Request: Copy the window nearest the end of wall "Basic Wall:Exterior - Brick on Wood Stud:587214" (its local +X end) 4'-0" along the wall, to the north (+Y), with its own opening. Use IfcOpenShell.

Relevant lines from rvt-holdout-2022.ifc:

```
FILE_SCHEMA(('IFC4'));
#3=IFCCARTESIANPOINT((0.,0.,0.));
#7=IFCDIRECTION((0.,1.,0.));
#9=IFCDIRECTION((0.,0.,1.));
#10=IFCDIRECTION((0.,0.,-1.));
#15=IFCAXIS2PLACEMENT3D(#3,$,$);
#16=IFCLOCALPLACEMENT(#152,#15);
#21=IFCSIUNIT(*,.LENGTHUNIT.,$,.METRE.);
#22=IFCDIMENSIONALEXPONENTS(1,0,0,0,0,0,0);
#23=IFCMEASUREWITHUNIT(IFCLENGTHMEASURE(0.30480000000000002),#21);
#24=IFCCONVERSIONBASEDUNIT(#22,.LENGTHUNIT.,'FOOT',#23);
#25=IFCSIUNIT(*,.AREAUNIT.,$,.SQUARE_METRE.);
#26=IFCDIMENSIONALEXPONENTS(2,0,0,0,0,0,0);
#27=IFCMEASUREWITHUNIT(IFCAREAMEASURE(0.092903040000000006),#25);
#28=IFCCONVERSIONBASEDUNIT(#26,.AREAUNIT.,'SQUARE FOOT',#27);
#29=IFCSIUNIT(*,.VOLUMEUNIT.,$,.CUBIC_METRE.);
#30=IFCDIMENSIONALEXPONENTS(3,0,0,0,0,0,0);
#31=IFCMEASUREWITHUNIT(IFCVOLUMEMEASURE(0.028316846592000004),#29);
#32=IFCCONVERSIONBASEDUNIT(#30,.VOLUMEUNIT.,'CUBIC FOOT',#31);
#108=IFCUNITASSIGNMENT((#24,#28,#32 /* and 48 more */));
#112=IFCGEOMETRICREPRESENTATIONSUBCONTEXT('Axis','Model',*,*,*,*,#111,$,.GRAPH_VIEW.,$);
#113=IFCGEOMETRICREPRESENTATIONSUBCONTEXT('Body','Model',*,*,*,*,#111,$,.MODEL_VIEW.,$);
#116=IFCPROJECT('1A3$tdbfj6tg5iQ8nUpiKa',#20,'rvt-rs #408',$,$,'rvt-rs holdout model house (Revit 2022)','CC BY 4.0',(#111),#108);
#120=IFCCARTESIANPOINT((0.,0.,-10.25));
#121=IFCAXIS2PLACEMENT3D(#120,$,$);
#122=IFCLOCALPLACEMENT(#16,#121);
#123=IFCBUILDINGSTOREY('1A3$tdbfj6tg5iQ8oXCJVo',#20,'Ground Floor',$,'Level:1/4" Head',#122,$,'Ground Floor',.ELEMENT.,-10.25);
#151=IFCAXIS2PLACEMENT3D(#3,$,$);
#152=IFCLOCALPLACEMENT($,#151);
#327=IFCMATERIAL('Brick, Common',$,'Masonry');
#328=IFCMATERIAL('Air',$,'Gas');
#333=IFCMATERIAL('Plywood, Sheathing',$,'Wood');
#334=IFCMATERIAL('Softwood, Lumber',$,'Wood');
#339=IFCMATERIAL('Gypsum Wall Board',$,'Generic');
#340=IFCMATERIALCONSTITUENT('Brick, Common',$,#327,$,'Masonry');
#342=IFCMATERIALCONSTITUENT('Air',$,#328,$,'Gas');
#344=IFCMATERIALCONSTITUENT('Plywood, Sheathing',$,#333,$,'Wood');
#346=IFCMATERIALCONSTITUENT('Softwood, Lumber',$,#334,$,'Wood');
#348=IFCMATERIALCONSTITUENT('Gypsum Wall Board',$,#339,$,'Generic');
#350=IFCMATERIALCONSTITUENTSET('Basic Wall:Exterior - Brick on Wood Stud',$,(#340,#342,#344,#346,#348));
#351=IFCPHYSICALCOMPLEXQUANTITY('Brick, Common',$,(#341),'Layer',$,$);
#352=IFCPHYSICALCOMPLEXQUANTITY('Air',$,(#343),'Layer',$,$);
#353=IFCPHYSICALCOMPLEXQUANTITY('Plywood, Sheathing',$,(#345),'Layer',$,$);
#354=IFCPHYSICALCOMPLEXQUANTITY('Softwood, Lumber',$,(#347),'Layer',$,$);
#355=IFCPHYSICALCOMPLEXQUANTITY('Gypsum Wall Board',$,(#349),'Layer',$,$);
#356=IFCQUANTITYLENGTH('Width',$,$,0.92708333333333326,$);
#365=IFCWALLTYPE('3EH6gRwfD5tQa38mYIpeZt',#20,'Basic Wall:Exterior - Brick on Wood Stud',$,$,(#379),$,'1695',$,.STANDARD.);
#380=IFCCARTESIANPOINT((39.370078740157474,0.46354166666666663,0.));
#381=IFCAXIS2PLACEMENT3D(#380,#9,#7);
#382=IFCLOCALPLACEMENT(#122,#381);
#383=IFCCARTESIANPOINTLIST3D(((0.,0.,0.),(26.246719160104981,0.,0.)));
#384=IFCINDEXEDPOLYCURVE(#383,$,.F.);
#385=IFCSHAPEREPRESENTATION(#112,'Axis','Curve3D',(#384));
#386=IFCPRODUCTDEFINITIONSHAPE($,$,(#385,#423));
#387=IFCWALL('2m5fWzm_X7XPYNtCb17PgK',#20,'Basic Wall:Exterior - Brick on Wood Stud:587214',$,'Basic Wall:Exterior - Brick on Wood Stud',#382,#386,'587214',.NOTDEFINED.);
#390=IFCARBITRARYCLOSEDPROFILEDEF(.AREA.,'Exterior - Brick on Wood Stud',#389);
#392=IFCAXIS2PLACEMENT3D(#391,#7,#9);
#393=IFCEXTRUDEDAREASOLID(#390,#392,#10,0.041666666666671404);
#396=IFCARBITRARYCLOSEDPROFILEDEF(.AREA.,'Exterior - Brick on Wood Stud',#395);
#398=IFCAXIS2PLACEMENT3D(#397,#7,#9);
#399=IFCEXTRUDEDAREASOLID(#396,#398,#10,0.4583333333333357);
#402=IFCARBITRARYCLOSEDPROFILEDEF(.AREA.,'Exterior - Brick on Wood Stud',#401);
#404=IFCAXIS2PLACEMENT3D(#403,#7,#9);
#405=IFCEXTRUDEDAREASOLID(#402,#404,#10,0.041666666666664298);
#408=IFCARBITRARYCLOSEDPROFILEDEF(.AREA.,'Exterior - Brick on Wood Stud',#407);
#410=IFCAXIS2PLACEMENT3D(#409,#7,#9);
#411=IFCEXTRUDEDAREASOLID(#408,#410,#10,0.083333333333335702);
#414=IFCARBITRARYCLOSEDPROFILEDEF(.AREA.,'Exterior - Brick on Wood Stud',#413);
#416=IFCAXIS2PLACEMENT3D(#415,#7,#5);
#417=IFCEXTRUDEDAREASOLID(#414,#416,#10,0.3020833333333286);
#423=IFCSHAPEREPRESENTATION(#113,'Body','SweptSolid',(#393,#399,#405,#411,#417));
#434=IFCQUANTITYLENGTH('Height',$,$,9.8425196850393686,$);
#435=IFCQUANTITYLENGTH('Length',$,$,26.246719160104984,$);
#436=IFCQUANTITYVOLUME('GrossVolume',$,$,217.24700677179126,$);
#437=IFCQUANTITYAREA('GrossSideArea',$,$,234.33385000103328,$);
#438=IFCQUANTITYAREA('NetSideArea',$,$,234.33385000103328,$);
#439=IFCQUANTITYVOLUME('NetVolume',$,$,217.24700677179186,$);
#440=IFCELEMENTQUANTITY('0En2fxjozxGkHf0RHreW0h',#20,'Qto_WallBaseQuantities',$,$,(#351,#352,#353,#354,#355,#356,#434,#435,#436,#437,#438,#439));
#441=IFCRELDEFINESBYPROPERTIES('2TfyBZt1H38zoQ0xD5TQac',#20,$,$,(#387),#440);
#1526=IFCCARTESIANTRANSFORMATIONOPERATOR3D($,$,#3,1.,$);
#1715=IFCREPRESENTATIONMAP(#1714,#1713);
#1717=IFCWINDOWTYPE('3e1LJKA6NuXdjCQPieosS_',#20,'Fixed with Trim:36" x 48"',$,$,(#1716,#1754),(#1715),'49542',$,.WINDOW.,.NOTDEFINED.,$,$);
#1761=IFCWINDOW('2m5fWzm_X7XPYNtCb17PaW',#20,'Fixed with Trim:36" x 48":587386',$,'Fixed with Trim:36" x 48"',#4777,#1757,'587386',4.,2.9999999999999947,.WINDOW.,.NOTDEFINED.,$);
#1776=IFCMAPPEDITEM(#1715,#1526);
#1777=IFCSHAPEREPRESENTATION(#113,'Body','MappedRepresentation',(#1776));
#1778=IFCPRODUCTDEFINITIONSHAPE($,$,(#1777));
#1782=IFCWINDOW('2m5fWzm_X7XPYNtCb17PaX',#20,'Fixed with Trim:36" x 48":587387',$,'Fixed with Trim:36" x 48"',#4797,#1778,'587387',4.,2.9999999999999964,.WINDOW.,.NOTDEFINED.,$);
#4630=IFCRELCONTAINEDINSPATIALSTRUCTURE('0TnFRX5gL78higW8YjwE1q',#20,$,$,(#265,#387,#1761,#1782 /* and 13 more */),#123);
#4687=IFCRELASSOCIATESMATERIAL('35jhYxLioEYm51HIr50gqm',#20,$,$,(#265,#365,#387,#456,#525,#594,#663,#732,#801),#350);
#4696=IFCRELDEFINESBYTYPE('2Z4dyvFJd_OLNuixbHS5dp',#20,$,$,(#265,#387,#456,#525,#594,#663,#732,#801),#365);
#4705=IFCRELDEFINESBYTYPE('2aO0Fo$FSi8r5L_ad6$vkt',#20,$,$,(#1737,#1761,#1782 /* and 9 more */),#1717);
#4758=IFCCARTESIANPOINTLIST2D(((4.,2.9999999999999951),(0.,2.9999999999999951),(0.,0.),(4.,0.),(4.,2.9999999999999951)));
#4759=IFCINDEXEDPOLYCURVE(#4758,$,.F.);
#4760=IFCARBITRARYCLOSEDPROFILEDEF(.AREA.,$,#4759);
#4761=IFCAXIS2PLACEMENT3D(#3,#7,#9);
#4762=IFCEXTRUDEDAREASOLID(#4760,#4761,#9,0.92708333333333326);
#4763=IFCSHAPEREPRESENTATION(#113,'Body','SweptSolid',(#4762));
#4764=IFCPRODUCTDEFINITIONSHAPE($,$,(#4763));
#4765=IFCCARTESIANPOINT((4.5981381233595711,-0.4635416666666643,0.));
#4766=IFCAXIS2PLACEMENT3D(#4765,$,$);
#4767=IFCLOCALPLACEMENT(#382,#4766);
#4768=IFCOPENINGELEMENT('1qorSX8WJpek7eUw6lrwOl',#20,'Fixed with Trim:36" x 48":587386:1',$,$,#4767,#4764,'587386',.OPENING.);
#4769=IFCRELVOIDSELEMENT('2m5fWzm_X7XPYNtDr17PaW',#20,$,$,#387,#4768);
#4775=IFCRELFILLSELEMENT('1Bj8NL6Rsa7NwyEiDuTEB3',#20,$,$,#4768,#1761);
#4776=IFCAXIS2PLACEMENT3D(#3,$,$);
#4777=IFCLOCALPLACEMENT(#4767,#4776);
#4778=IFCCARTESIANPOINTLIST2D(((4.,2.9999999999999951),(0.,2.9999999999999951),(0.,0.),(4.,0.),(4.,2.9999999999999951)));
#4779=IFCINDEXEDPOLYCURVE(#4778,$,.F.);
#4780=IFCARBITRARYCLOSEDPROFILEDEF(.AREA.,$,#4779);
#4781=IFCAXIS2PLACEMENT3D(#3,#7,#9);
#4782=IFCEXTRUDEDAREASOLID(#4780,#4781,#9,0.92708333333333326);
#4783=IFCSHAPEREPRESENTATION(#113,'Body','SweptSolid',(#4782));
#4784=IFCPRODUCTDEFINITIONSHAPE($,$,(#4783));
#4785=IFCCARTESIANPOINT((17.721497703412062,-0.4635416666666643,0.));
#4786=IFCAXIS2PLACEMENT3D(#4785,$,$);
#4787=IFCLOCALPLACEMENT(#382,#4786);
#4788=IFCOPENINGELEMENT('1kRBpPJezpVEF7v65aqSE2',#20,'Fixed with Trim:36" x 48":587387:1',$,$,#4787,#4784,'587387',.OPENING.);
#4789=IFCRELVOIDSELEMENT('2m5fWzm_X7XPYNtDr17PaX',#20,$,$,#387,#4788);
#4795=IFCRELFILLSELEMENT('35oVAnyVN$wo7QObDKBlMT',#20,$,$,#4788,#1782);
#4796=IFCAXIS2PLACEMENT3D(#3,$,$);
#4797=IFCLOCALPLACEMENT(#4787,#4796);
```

```python
import ifcopenshell
import ifcopenshell.api.feature
import ifcopenshell.api.geometry
import ifcopenshell.api.pset
import ifcopenshell.api.root
import ifcopenshell.geom
import ifcopenshell.util.element
import ifcopenshell.util.placement
import ifcopenshell.util.shape
import ifcopenshell.util.unit

model = ifcopenshell.open("rvt-holdout-2022.ifc")
unit_scale = ifcopenshell.util.unit.calculate_unit_scale(model)
area_scale = ifcopenshell.util.unit.calculate_unit_scale(model, "AREAUNIT")
volume_scale = ifcopenshell.util.unit.calculate_unit_scale(model, "VOLUMEUNIT")
settings = ifcopenshell.geom.settings()


def volume(element):
    """Net volume in cubic metres, openings subtracted."""
    shape = ifcopenshell.geom.create_shape(settings, element)
    return ifcopenshell.util.shape.get_volume(shape.geometry)


def reuse_history(source, copy):
    """copy_class also copies each property set's owner history, people and application; keep the originals."""
    for rel in copy.IsDefinedBy:
        if rel.is_a("IfcRelDefinesByProperties") and (history := rel.RelatingPropertyDefinition.OwnerHistory):
            rel.RelatingPropertyDefinition.OwnerHistory = source.OwnerHistory
            ifcopenshell.util.element.remove_deep2(model, history)


window = model.by_guid("2m5fWzm_X7XPYNtCb17PaX")
opening = window.FillsVoids[0].RelatingOpeningElement
wall = opening.VoidsElements[0].RelatingBuildingElement
before = volume(wall)
shift = ifcopenshell.util.placement.get_local_placement(wall.ObjectPlacement)[:3, 0] * 48 * 0.0254 / unit_scale

# copy_class copies the void relationship, type, container and properties, but no geometry.
new_opening = ifcopenshell.api.root.copy_class(model, product=opening)
new_opening.Representation = ifcopenshell.util.element.copy_deep(
    model, opening.Representation, exclude=["IfcGeometricRepresentationContext", "IfcRepresentationMap"]
)
new_opening.Name = 'Fixed with Trim:36" x 48"'
new_opening.Tag = None
reuse_history(opening, new_opening)
new_window = ifcopenshell.api.root.copy_class(model, product=window)
new_window.Representation = ifcopenshell.util.element.copy_deep(
    model, window.Representation, exclude=["IfcGeometricRepresentationContext", "IfcRepresentationMap"]
)
new_window.Name = 'Fixed with Trim:36" x 48"'
new_window.Tag = None
reuse_history(window, new_window)
ifcopenshell.api.feature.add_filling(model, opening=new_opening, element=new_window)

for old, new in ((opening, new_opening), (window, new_window)):
    matrix = ifcopenshell.util.placement.get_local_placement(old.ObjectPlacement)
    matrix[:3, 3] += shift
    ifcopenshell.api.geometry.edit_object_placement(model, product=new, matrix=matrix, is_si=False)

after = volume(wall)
thickness = 0.2826  # wall thickness in metres

# Update the wall's stored quantities.
qto = model.by_id(ifcopenshell.util.element.get_pset(wall, "Qto_WallBaseQuantities", should_inherit=False)["id"])
ifcopenshell.api.pset.edit_qto(model, qto=qto, properties={
    "NetSideArea": after / thickness / area_scale,
    "NetVolume": after / volume_scale,
})

print(f"wall volume {before:.3f} -> {after:.3f} m3")

model.write("rvt-holdout-2022_v2.ifc")
```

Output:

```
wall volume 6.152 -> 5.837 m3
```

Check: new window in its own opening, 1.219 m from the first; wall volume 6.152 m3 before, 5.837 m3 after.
